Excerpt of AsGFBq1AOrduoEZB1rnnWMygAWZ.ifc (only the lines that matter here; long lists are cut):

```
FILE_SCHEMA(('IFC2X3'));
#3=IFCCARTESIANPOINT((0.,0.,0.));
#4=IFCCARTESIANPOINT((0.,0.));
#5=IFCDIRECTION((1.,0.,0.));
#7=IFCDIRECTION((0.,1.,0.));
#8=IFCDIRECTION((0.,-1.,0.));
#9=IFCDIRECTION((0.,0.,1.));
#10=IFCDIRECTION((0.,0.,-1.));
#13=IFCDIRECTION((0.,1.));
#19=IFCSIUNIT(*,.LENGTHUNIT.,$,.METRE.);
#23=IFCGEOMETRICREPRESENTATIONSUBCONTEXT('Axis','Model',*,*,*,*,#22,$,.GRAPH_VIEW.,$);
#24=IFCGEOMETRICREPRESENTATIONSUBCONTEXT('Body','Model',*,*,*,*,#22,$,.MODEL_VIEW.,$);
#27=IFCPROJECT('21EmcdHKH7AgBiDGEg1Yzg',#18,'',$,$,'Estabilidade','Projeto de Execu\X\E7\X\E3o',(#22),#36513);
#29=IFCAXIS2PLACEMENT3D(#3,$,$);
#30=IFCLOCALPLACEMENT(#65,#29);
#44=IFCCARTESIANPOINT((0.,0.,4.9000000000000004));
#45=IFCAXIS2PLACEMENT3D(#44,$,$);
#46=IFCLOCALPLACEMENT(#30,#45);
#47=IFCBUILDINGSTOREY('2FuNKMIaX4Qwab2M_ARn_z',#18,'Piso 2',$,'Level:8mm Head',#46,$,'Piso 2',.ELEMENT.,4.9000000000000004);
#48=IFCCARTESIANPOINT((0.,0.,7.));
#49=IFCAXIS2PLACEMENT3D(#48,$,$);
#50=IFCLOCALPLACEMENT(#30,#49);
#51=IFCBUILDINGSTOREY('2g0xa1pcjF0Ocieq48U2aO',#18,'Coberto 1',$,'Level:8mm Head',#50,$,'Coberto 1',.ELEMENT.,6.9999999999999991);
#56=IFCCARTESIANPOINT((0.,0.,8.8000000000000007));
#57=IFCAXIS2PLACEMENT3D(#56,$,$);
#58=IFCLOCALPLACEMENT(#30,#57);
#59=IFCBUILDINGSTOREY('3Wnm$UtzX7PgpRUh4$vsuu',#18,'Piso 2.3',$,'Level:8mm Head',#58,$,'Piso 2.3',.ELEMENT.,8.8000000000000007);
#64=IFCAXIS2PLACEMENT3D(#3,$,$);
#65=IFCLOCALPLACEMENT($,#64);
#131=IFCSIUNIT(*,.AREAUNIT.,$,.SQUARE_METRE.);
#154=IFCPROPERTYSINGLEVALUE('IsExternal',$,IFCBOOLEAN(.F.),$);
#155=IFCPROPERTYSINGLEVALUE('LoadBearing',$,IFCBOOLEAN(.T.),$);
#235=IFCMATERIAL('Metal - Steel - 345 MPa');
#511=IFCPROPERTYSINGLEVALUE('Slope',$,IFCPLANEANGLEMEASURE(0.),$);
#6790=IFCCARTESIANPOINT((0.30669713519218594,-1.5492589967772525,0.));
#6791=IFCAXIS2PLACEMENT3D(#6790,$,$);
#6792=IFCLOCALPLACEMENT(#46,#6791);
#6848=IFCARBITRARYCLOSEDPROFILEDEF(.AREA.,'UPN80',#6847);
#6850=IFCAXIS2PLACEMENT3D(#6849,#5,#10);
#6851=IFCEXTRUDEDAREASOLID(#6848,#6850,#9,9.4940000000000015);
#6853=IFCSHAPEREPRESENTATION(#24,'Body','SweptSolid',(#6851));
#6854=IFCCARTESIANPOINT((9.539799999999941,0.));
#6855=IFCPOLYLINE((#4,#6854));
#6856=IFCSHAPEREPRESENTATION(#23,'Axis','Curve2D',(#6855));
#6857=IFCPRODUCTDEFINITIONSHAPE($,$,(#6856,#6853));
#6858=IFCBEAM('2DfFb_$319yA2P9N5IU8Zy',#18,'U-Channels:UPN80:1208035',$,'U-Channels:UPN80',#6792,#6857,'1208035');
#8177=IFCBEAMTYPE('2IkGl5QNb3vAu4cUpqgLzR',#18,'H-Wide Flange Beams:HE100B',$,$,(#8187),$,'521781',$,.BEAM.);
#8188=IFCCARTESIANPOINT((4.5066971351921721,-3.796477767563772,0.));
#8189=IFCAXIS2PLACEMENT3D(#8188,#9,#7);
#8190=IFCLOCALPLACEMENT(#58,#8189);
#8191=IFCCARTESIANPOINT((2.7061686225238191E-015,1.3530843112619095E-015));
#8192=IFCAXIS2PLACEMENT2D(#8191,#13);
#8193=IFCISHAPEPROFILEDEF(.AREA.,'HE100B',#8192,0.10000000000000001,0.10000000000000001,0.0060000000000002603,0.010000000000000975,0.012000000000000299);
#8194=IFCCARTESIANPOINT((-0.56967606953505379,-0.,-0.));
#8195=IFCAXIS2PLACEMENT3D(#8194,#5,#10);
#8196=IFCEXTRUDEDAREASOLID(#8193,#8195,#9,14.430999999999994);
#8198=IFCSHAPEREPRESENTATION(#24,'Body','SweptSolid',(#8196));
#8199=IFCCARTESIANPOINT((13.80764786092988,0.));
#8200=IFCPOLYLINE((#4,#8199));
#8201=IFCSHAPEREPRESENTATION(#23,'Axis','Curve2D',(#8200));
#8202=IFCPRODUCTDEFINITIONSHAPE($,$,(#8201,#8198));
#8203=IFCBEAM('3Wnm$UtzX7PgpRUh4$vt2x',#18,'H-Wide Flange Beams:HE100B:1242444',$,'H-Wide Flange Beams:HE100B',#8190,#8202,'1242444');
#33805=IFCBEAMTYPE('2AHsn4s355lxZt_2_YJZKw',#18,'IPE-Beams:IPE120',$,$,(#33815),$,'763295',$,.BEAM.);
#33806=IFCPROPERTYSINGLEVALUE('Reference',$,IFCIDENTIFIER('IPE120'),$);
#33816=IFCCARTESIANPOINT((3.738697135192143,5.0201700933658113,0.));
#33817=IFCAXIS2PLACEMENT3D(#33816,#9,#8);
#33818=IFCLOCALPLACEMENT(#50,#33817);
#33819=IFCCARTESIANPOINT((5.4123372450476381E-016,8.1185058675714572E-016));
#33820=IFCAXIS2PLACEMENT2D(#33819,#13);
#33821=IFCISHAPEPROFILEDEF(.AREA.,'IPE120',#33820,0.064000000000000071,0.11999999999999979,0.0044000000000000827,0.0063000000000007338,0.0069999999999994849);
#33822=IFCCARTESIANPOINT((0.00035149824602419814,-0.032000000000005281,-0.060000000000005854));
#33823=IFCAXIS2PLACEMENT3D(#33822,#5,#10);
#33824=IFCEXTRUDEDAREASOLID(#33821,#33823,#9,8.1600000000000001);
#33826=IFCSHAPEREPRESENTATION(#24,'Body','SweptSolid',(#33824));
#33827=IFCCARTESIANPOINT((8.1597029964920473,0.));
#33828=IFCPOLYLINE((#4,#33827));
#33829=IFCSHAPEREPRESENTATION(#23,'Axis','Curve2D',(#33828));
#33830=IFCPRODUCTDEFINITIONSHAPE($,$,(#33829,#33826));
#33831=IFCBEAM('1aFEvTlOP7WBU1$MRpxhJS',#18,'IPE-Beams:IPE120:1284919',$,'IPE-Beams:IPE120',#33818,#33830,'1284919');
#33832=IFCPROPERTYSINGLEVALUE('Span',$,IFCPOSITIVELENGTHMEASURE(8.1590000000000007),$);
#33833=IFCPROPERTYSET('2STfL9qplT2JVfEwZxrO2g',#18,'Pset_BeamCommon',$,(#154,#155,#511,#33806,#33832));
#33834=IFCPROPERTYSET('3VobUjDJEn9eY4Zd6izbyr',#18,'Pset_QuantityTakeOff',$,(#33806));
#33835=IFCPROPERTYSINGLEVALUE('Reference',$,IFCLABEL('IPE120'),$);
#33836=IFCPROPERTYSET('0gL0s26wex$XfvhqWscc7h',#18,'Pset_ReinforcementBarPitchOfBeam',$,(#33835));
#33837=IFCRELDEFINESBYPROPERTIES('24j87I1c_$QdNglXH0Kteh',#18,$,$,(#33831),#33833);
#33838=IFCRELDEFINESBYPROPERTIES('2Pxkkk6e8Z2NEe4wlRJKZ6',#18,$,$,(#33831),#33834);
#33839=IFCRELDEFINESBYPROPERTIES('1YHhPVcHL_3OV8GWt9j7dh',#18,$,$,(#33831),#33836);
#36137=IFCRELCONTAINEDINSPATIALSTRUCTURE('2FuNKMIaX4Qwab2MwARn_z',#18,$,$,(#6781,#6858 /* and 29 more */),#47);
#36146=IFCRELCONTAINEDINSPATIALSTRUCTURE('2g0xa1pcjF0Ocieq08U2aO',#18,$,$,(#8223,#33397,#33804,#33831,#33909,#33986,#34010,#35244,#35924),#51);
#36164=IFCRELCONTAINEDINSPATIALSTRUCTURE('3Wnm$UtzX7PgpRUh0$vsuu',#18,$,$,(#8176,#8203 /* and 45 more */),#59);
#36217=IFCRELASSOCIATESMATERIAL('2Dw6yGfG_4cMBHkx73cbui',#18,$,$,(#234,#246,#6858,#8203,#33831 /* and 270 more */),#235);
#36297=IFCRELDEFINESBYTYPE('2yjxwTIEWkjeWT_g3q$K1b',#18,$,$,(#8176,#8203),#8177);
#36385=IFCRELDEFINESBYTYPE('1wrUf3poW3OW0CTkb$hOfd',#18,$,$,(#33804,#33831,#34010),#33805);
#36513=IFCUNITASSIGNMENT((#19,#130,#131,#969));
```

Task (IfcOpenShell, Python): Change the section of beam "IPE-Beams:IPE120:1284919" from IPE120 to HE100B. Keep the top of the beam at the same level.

```python
import ifcopenshell
import ifcopenshell.api.pset
import ifcopenshell.api.type
import ifcopenshell.util.element
import ifcopenshell.util.representation

model = ifcopenshell.open("AsGFBq1AOrduoEZB1rnnWMygAWZ.ifc")

member = model.by_guid("1aFEvTlOP7WBU1$MRpxhJS")
source = next(p for p in model.by_type("IfcIShapeProfileDef") if p.ProfileName == "HE100B")

body = ifcopenshell.util.representation.get_representation(member, "Model", "Body")
solid = body.Items[0]
old_profile = solid.SweptArea

# Copy the section's sizes but keep this member's own profile position.
profile = ifcopenshell.util.element.copy(model, source)
# Profiles are centred, so shift by half the change in depth to hold the top.
shift = (old_profile.OverallDepth - profile.OverallDepth) / 2
x, y = old_profile.Position.Location.Coordinates
up = (-1.0, 0.0)  # upwards, in the solid's own plane
location = model.createIfcCartesianPoint((x + up[0] * shift, y + up[1] * shift))
profile.Position = model.createIfcAxis2Placement2D(location, old_profile.Position.RefDirection)
solid.SweptArea = profile
if not model.get_total_inverses(old_profile):
    ifcopenshell.util.element.remove_deep2(model, old_profile)

new_type = model.by_id(8177)
ifcopenshell.api.type.assign_type(
    model, related_objects=[member], relating_type=new_type, should_map_representations=False
)
member.Name = member.Name.replace("IPE120", "HE100B")
member.ObjectType = "IPE-Beams:HE100B"
pset = model.by_id(ifcopenshell.util.element.get_pset(member, "Pset_BeamCommon", should_inherit=False)["id"])
ifcopenshell.api.pset.edit_pset(model, pset=pset, properties={"Reference": "HE100B"})
pset = model.by_id(ifcopenshell.util.element.get_pset(member, "Pset_QuantityTakeOff", should_inherit=False)["id"])
ifcopenshell.api.pset.edit_pset(model, pset=pset, properties={"Reference": "HE100B"})
pset = model.by_id(ifcopenshell.util.element.get_pset(member, "Pset_ReinforcementBarPitchOfBeam", should_inherit=False)["id"])
ifcopenshell.api.pset.edit_pset(model, pset=pset, properties={"Reference": "HE100B"})

print(solid.SweptArea)

model.write("AsGFBq1AOrduoEZB1rnnWMygAWZ_edited.ifc")
```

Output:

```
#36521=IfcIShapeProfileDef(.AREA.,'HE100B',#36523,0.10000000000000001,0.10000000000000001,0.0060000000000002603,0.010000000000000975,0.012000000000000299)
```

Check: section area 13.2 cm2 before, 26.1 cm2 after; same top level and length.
